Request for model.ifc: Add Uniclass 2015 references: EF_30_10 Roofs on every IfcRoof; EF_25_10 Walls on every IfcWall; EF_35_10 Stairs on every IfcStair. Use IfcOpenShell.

First a look at what the model holds.

```python
import ifcopenshell

model = ifcopenshell.open("model.ifc")
print(model.schema)
print("classifications:", [c.Name for c in model.by_type("IfcClassification")])
for ifc_class in ("IfcDoor", "IfcRoof", "IfcStair", "IfcWall", "IfcWindow"):
    print(ifc_class, len(model.by_type(ifc_class)))
```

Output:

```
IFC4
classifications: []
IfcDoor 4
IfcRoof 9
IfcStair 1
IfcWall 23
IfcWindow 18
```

```python
import ifcopenshell
import ifcopenshell.api.classification

model = ifcopenshell.open("model.ifc")

system = ifcopenshell.api.classification.add_classification(model, classification="Uniclass 2015")

codes = {
    "IfcRoof": ("EF_30_10", "Roofs"),
    "IfcWall": ("EF_25_10", "Walls"),
    "IfcStair": ("EF_35_10", "Stairs"),
}
for ifc_class, (code, name) in codes.items():
    products = model.by_type(ifc_class)
    ifcopenshell.api.classification.add_reference(
        model, products=products, classification=system, identification=code, name=name
    )
    print(code, len(products))

model.write("model_rev.ifc")
```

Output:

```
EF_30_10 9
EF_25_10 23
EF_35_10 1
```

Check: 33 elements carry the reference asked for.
